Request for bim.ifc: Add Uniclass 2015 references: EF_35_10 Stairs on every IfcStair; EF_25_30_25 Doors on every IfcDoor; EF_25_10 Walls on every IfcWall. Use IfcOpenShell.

First a look at what the model holds.

```python
import ifcopenshell

model = ifcopenshell.open("bim.ifc")
print(model.schema)
print("classifications:", [c.Name for c in model.by_type("IfcClassification")])
for ifc_class in ("IfcDoor", "IfcRoof", "IfcStair", "IfcWall", "IfcWindow"):
    print(ifc_class, len(model.by_type(ifc_class)))
```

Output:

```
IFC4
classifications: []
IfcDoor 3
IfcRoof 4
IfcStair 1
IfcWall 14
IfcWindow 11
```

```python
import ifcopenshell
import ifcopenshell.api.classification

model = ifcopenshell.open("bim.ifc")

system = ifcopenshell.api.classification.add_classification(model, classification="Uniclass 2015")

codes = {
    "IfcStair": ("EF_35_10", "Stairs"),
    "IfcDoor": ("EF_25_30_25", "Doors"),
    "IfcWall": ("EF_25_10", "Walls"),
}
for ifc_class, (code, name) in codes.items():
    products = model.by_type(ifc_class)
    ifcopenshell.api.classification.add_reference(
        model, products=products, classification=system, identification=code, name=name
    )
    print(code, len(products))

model.write("bim_edited.ifc")
```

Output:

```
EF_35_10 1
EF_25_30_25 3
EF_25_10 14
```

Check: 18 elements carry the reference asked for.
